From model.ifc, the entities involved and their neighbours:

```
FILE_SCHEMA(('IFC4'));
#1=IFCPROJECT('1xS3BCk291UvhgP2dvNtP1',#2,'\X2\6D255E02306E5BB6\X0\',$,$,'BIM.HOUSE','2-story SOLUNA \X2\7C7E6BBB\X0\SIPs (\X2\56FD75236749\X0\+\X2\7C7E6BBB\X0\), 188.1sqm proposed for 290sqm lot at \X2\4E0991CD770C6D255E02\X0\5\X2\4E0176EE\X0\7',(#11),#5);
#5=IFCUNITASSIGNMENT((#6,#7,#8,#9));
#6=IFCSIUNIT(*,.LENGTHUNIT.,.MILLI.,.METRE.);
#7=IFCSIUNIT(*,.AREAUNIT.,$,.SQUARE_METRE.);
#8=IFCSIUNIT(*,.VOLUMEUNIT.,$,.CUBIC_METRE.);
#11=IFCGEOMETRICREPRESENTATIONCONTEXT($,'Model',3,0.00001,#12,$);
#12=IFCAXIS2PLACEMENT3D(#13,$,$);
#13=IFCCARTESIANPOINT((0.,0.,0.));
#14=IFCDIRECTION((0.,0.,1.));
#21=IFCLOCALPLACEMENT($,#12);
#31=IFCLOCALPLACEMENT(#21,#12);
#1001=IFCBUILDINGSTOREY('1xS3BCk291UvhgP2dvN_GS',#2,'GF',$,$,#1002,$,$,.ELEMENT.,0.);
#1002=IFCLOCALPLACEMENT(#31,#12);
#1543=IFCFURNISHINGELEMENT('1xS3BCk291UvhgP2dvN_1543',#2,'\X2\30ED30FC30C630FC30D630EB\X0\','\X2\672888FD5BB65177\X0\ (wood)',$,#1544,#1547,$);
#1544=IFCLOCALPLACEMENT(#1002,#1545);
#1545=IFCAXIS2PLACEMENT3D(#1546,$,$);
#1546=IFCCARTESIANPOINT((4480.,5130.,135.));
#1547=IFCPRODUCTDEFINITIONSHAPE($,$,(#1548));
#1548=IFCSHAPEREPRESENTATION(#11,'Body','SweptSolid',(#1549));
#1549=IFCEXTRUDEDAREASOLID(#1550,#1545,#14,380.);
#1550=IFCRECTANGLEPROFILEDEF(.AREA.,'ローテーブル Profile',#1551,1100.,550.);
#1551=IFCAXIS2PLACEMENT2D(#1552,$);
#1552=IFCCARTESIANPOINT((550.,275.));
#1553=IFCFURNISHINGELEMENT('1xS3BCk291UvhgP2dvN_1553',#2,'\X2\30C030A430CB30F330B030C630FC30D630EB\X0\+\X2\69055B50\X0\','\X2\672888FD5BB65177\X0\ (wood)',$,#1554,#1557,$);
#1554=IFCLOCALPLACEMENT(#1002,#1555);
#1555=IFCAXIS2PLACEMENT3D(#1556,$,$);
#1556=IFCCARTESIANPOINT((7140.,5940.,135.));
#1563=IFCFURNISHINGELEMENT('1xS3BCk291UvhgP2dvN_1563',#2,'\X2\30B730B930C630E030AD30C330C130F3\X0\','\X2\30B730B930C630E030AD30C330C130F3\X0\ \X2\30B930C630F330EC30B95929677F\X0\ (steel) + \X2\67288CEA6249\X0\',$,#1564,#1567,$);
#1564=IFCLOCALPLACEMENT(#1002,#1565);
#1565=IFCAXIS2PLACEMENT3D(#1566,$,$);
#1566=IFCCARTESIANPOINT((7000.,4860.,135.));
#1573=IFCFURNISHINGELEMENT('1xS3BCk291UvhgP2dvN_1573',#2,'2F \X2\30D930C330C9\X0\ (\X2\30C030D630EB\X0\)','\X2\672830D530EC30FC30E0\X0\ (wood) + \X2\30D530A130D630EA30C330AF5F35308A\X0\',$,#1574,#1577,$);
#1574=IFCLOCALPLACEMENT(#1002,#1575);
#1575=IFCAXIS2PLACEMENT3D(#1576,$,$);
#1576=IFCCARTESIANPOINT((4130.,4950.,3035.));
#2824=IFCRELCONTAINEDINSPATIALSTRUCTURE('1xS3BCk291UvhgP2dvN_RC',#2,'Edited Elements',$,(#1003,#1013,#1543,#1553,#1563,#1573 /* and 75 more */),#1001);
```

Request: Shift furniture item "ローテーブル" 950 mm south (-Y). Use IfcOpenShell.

```python
import ifcopenshell
import ifcopenshell.api.geometry
import ifcopenshell.util.placement

model = ifcopenshell.open("model.ifc")

item = model.by_guid("1xS3BCk291UvhgP2dvN_1543")
matrix = ifcopenshell.util.placement.get_local_placement(item.ObjectPlacement)
matrix[1, 3] -= 950.0
ifcopenshell.api.geometry.edit_object_placement(model, product=item, matrix=matrix, is_si=False)

print(ifcopenshell.util.placement.get_local_placement(item.ObjectPlacement).round(3) + 0.0)

model.write("model_v2.ifc")
```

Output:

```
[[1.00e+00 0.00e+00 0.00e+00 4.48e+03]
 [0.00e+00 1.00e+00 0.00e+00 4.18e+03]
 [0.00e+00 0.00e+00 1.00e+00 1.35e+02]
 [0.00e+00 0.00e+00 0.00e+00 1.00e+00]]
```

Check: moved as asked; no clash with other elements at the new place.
